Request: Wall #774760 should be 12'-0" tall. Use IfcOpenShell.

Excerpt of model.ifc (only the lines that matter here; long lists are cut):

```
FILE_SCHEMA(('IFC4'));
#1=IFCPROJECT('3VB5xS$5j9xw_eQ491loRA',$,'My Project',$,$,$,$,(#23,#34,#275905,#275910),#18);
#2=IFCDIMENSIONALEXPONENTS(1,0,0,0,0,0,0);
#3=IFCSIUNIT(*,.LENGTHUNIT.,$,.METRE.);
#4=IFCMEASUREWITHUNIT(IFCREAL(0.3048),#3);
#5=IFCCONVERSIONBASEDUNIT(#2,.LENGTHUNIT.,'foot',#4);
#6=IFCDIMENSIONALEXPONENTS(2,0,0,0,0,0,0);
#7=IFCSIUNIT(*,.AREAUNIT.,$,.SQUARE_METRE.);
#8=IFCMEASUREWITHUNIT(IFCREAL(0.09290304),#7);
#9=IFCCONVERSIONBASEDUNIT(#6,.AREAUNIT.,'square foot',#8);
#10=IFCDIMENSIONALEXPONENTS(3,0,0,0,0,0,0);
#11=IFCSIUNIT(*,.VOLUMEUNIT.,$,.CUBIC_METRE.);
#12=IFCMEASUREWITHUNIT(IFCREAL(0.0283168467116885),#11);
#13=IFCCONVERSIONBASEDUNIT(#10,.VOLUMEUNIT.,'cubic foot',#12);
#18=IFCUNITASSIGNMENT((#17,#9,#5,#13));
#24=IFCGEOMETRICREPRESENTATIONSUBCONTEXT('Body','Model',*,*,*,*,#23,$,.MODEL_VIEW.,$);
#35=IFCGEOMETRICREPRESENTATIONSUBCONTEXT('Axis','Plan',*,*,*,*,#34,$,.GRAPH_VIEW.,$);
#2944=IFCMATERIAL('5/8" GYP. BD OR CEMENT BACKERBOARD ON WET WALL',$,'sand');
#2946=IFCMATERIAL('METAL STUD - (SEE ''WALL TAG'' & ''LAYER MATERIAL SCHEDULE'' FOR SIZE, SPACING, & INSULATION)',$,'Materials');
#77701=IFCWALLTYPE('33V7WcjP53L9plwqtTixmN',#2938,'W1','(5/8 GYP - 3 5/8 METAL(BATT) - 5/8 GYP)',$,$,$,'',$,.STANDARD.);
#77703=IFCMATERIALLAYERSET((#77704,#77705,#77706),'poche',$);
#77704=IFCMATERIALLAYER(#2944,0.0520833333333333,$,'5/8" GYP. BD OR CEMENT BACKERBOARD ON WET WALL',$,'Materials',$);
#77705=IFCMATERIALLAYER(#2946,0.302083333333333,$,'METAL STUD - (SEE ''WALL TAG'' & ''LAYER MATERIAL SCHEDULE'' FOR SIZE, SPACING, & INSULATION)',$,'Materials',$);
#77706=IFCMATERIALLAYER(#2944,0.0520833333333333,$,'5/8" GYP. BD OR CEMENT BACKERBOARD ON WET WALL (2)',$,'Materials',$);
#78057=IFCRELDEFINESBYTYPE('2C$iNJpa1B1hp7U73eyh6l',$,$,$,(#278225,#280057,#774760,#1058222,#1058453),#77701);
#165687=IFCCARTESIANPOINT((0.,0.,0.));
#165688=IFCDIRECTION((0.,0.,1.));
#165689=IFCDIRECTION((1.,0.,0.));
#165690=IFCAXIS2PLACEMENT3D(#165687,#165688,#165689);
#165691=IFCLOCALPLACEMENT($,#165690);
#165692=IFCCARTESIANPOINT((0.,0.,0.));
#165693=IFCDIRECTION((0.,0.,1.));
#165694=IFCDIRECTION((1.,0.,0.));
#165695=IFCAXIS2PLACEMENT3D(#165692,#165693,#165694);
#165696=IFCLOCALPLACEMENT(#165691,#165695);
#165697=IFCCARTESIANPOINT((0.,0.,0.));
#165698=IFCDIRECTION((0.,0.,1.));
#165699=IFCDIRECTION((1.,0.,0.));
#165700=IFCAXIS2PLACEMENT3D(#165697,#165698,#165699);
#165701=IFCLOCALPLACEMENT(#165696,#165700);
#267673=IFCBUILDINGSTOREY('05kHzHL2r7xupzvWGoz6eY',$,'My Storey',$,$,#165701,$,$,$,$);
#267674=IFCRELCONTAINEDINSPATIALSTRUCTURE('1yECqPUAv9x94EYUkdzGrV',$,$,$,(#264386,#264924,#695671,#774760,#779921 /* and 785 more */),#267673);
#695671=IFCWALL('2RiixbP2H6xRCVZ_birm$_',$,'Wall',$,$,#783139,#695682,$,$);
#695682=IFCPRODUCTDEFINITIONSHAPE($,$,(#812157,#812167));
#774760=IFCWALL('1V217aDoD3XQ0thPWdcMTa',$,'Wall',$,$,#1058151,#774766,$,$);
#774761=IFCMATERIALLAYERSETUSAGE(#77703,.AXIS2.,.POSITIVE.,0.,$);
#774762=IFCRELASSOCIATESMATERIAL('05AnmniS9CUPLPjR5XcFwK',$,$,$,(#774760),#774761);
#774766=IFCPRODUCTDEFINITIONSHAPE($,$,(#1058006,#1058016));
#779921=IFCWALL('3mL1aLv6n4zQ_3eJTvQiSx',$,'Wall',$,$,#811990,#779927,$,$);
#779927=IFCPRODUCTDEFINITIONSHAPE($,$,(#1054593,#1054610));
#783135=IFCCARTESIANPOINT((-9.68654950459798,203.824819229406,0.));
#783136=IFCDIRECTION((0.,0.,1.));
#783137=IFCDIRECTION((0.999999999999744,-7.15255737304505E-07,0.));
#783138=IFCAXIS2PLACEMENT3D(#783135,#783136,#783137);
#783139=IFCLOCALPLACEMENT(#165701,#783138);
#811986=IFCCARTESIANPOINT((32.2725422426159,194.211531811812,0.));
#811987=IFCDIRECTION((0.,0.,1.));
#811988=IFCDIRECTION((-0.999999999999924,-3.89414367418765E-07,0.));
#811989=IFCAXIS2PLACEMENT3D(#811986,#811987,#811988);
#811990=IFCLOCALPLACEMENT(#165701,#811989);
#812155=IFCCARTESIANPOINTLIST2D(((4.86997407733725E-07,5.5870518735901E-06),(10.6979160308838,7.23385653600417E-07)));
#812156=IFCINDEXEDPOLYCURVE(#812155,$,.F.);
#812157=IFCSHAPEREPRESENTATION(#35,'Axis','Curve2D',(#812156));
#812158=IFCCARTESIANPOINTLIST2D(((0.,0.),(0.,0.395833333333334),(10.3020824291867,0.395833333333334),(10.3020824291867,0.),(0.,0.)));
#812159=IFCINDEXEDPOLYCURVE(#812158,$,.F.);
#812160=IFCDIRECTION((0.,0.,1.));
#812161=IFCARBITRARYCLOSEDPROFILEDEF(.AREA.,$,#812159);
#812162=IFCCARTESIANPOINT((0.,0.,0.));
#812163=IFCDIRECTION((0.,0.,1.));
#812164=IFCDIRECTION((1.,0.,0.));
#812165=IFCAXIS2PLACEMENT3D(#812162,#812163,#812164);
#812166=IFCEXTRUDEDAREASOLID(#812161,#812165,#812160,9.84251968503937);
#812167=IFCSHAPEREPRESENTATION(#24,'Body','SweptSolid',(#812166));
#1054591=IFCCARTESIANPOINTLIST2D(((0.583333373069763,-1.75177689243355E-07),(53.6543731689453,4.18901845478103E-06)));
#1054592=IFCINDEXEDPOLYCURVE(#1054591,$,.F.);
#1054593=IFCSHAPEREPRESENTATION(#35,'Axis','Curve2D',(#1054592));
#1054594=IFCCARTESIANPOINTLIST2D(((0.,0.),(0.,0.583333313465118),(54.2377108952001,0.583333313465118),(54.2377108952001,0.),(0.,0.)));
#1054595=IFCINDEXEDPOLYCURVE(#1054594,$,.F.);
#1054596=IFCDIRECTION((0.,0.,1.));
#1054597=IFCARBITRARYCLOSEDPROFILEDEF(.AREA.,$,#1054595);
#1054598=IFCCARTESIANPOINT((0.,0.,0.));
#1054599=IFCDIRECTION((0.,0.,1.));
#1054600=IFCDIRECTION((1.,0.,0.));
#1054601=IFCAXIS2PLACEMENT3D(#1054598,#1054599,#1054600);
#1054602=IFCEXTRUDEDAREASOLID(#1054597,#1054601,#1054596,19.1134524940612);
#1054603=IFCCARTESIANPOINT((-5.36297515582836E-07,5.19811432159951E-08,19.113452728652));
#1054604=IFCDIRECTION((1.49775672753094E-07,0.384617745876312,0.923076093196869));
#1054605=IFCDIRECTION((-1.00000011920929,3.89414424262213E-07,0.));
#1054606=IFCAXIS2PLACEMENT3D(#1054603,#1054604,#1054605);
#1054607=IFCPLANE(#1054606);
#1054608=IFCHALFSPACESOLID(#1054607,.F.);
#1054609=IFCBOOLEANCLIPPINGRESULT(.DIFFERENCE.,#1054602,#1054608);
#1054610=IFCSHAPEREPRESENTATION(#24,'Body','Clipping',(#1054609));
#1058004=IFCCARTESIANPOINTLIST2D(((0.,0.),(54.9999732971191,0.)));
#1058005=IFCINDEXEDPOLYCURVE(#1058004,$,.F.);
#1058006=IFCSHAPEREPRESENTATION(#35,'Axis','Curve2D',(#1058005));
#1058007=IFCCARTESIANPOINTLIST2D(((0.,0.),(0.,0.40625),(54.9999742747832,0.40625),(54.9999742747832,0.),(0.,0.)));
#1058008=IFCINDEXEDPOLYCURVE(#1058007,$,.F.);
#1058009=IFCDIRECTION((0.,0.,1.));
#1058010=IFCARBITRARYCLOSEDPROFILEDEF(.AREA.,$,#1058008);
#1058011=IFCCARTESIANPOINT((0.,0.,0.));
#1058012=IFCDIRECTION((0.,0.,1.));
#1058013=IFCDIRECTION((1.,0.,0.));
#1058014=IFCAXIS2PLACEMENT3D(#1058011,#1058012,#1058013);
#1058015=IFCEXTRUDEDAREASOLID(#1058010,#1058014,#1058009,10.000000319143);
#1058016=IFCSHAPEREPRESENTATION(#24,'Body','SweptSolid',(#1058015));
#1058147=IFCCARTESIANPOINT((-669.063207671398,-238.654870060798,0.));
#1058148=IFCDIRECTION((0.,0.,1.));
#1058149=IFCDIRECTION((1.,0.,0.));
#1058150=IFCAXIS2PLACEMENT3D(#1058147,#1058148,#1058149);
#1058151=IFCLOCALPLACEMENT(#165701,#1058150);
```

```python
import ifcopenshell
import ifcopenshell.geom
import ifcopenshell.util.representation
import ifcopenshell.util.shape
import ifcopenshell.util.unit

model = ifcopenshell.open("model.ifc")
unit_scale = ifcopenshell.util.unit.calculate_unit_scale(model)
settings = ifcopenshell.geom.settings()


def volume(element):
    """Net volume in cubic metres, openings subtracted."""
    shape = ifcopenshell.geom.create_shape(settings, element)
    return ifcopenshell.util.shape.get_volume(shape.geometry)


wall = model.by_guid("1V217aDoD3XQ0thPWdcMTa")
before = volume(wall)

body = ifcopenshell.util.representation.get_representation(wall, "Model", "Body")
solid = body.Items[0]
old_height = solid.Depth
solid.Depth = 144 * 0.0254 / unit_scale
after = volume(wall)

print(f"height {old_height:g} -> {solid.Depth:g}, volume {before:.3f} -> {after:.3f} m3")

model.write("model_v2.ifc")
```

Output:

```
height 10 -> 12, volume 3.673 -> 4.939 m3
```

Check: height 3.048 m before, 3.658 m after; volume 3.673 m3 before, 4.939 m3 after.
